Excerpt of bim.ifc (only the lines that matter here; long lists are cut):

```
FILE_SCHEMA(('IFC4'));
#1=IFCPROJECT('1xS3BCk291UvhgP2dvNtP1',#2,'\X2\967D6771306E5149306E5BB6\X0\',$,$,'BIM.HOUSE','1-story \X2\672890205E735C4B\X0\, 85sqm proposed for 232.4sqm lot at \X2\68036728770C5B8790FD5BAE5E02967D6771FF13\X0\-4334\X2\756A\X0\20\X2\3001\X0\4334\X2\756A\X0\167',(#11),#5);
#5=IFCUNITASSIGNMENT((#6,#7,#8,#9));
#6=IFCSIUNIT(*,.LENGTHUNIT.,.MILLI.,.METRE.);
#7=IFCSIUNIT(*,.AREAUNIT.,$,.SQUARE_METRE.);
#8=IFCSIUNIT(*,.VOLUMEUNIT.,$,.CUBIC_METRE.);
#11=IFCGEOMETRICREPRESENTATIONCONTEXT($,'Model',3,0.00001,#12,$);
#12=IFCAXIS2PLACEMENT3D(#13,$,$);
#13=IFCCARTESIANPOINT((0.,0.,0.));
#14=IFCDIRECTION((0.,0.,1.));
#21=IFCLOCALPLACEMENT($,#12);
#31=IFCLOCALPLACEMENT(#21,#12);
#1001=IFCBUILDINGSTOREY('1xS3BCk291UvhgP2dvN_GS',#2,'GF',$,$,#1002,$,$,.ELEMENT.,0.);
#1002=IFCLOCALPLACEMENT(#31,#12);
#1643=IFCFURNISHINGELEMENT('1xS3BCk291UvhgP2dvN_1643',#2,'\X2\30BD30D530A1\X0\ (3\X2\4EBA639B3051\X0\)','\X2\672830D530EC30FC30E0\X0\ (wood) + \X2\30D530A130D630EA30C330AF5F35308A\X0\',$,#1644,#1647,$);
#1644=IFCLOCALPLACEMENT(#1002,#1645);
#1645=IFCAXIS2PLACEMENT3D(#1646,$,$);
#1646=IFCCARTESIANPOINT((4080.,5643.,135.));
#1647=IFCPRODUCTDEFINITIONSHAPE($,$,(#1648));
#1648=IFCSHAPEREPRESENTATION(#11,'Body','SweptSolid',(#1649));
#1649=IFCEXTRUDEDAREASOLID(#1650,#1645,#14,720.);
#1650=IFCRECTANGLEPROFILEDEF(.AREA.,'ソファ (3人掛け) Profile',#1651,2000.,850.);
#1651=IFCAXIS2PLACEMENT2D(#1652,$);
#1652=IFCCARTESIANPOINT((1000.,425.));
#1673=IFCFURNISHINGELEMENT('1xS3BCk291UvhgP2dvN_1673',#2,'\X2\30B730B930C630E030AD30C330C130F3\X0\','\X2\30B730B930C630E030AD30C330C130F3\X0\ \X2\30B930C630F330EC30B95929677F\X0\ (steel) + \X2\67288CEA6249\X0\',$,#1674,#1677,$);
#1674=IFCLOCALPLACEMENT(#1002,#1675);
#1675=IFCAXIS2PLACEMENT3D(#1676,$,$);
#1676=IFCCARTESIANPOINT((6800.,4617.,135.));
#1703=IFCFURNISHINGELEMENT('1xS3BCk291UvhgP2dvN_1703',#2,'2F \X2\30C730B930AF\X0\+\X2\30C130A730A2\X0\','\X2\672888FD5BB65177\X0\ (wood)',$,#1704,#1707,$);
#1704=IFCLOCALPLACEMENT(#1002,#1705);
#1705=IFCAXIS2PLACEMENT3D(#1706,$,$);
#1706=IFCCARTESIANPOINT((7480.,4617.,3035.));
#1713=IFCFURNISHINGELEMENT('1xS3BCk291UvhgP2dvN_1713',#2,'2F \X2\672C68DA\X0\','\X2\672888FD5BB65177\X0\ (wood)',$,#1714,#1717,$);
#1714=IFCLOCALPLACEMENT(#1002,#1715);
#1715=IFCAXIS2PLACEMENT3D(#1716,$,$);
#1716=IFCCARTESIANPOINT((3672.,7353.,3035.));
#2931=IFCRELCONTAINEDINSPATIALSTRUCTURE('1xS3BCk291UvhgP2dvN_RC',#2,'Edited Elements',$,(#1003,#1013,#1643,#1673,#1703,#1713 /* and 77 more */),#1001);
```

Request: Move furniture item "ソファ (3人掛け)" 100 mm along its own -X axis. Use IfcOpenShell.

```python
import ifcopenshell
import ifcopenshell.api.geometry
import ifcopenshell.util.placement

model = ifcopenshell.open("bim.ifc")

item = model.by_id(1643)
matrix = ifcopenshell.util.placement.get_local_placement(item.ObjectPlacement)
matrix[:3, 3] -= matrix[:3, 0] * 100.0
ifcopenshell.api.geometry.edit_object_placement(model, product=item, matrix=matrix, is_si=False)

print(ifcopenshell.util.placement.get_local_placement(item.ObjectPlacement).round(3) + 0.0)

model.write("bim_v2.ifc")
```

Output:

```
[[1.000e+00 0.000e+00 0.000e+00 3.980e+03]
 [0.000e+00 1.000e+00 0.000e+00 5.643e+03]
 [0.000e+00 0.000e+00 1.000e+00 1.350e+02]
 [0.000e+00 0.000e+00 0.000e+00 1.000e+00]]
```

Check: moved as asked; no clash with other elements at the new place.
